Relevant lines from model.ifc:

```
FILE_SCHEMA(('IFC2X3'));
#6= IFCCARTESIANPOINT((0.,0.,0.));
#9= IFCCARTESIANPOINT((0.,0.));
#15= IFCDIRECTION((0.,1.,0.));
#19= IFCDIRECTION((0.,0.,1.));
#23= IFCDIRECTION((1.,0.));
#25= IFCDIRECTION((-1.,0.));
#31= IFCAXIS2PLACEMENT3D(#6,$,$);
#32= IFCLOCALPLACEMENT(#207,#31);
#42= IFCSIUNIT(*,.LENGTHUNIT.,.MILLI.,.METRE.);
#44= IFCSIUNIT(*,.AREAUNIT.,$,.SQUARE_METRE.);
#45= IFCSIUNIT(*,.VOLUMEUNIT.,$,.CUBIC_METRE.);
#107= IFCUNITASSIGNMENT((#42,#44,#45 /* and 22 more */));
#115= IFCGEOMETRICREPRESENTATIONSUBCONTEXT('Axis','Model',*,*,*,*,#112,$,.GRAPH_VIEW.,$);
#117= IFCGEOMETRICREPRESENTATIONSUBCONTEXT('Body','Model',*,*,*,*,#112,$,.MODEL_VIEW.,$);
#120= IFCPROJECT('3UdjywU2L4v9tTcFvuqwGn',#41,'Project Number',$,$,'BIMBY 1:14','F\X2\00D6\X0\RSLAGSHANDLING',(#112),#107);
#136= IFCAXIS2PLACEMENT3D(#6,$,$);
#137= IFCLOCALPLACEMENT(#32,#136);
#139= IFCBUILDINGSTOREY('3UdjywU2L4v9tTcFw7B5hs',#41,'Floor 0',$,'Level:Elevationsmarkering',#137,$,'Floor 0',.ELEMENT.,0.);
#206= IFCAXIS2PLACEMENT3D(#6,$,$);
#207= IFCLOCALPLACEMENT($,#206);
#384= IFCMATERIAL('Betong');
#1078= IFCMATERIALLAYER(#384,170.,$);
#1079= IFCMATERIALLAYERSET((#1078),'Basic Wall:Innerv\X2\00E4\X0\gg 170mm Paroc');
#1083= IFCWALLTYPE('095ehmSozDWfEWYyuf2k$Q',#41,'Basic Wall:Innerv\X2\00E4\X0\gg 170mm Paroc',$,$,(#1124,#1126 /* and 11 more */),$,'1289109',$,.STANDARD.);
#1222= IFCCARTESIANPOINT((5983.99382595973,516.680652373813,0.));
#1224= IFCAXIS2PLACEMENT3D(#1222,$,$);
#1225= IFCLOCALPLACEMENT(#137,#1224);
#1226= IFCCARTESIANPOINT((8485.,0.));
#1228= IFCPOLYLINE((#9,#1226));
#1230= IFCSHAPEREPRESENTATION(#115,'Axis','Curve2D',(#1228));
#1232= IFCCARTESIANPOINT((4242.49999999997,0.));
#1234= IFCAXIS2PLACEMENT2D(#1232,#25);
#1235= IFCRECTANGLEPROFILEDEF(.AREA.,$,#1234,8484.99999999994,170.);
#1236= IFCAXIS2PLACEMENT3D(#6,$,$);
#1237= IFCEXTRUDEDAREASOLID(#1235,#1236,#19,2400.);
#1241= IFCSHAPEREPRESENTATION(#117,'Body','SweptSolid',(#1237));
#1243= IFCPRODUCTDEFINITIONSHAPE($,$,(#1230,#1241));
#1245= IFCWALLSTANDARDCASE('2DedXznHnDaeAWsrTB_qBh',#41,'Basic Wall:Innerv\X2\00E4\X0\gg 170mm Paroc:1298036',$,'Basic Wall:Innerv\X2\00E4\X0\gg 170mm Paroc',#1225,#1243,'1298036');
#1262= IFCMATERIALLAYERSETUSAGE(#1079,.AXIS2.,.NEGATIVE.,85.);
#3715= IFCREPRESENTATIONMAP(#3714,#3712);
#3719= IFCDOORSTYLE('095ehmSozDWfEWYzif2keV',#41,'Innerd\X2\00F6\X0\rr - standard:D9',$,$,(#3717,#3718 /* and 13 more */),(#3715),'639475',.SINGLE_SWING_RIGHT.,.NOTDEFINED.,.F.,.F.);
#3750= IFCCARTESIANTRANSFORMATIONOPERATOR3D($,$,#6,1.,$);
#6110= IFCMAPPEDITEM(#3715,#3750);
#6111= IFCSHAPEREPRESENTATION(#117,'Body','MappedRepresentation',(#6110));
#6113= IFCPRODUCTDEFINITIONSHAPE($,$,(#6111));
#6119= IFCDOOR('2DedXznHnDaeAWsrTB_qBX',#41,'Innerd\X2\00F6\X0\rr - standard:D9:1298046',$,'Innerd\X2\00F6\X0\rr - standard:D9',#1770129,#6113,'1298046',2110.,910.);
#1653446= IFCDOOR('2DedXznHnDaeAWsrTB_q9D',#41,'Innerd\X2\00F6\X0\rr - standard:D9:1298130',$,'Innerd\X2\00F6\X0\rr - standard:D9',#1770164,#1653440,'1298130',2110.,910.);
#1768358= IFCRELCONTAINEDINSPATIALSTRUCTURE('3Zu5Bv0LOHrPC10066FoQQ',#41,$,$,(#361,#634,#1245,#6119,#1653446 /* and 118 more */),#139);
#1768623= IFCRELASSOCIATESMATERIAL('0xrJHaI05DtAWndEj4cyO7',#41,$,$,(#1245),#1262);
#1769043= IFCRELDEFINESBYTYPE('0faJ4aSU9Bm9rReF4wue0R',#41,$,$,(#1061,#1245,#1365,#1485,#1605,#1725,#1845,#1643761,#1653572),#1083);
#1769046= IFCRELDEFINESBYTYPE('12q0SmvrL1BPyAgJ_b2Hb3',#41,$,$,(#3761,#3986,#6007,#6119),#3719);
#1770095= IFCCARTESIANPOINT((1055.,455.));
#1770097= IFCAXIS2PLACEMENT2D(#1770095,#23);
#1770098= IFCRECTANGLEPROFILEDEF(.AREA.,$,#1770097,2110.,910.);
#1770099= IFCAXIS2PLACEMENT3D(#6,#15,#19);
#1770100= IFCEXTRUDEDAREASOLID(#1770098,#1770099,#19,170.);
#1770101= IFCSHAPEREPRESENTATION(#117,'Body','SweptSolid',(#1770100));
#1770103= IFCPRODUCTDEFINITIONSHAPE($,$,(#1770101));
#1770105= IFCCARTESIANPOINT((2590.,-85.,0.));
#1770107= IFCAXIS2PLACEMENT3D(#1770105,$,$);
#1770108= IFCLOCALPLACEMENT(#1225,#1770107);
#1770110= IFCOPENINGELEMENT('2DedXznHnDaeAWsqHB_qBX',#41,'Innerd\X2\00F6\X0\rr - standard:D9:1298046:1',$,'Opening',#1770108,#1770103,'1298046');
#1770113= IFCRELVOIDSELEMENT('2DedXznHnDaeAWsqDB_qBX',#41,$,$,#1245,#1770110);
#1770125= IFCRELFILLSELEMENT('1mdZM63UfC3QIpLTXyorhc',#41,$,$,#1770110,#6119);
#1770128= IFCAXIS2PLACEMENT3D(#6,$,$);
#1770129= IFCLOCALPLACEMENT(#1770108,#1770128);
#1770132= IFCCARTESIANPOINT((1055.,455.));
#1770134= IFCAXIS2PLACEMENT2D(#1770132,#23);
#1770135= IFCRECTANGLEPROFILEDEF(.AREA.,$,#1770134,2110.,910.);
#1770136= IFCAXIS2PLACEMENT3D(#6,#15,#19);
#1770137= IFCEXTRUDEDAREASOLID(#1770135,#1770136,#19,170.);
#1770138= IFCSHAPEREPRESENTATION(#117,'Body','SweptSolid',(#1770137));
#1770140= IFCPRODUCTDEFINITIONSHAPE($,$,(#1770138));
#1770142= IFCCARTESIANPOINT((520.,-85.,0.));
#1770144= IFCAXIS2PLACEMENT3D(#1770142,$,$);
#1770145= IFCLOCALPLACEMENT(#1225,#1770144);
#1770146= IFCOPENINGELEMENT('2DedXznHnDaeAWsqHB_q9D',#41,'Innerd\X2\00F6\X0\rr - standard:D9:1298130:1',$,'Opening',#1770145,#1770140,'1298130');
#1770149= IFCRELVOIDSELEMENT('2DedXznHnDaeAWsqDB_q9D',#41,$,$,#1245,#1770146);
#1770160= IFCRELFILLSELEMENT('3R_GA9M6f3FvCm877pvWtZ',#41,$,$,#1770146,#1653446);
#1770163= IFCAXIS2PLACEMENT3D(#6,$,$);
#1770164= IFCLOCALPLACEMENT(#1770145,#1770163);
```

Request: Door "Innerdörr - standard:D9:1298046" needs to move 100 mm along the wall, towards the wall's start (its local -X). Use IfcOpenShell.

```python
import ifcopenshell
import ifcopenshell.api.geometry
import ifcopenshell.util.placement
import ifcopenshell.util.unit

model = ifcopenshell.open("model.ifc")
unit_scale = ifcopenshell.util.unit.calculate_unit_scale(model)

door = model.by_id(6119)
opening = door.FillsVoids[0].RelatingOpeningElement
wall = opening.VoidsElements[0].RelatingBuildingElement

wall_matrix = ifcopenshell.util.placement.get_local_placement(wall.ObjectPlacement)
shift = wall_matrix[:3, 0] * -0.1 / unit_scale
before = ifcopenshell.util.placement.get_local_placement(door.ObjectPlacement)[:3, 3].copy()

# The door is placed relative to its opening, so it follows when the opening moves.
matrix = ifcopenshell.util.placement.get_local_placement(opening.ObjectPlacement)
matrix[:3, 3] += shift
ifcopenshell.api.geometry.edit_object_placement(
    model, product=opening, matrix=matrix, is_si=False, should_transform_children=True
)

after = ifcopenshell.util.placement.get_local_placement(door.ObjectPlacement)[:3, 3]
print("door moved by", (after - before).round(3) + 0.0)

model.write("model_updated.ifc")
```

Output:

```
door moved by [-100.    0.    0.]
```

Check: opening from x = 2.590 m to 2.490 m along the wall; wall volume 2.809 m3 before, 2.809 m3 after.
